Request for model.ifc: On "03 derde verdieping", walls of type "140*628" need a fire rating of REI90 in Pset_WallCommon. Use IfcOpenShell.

First a look at what the model holds.

```python
import ifcopenshell
import ifcopenshell.util.element

model = ifcopenshell.open("model.ifc")
print(model.schema)
storey = next(s for s in model.by_type("IfcBuildingStorey") if s.Name == "03 derde verdieping")
walls = [e for e in ifcopenshell.util.element.get_decomposition(storey) if e.is_a("IfcWall")]
seen = {}
for e in walls:
    element_type = ifcopenshell.util.element.get_type(e)
    key = (element_type.Name if element_type != e and element_type else None, ifcopenshell.util.element.get_pset(e, "Pset_WallCommon", "FireRating"))
    seen[key] = seen.get(key, 0) + 1
for (name, value), count in sorted(seen.items(), key=str):
    print(count, "x", name, "|", value)
```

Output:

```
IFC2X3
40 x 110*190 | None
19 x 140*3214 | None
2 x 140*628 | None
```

```python
import ifcopenshell
import ifcopenshell.api.pset
import ifcopenshell.util.element

model = ifcopenshell.open("model.ifc")

storey = next(s for s in model.by_type("IfcBuildingStorey") if s.Name == "03 derde verdieping")
walls = [e for e in ifcopenshell.util.element.get_decomposition(storey) if e.is_a("IfcWall")]

count = 0
for e in walls:
    element_type = ifcopenshell.util.element.get_type(e)
    if element_type in (None, e) or element_type.Name != "140*628":
        continue
    found = ifcopenshell.util.element.get_pset(e, "Pset_WallCommon", should_inherit=False)
    if found:
        pset = model.by_id(found["id"])
        if len(ifcopenshell.util.element.get_elements_by_pset(pset)) > 1:
            pset = ifcopenshell.api.pset.unshare_pset(model, products=[e], pset=pset)[0]
    else:
        pset = ifcopenshell.api.pset.add_pset(model, product=e, name="Pset_WallCommon")
    ifcopenshell.api.pset.edit_pset(model, pset=pset, properties={"FireRating": "REI90"})
    count += 1

print(count, "walls updated")

model.write("model_rev.ifc")
```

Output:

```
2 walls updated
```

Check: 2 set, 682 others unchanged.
